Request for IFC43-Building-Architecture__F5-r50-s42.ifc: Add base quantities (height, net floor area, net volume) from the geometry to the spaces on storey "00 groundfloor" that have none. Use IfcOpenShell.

First a look at what the model holds.

```python
import ifcopenshell
import ifcopenshell.util.element
import ifcopenshell.util.unit

model = ifcopenshell.open("IFC43-Building-Architecture__F5-r50-s42.ifc")
print(model.schema)
for unit_type in ("LENGTHUNIT", "AREAUNIT", "VOLUMEUNIT"):
    print(unit_type, ifcopenshell.util.unit.calculate_unit_scale(model, unit_type))
storey = next(s for s in model.by_type("IfcBuildingStorey") if s.Name == "00 groundfloor")
spaces = [e for e in ifcopenshell.util.element.get_decomposition(storey) if e.is_a("IfcSpace")]
for e in sorted(spaces, key=lambda e: e.id()):
    print(e.id(), e.is_a(), e.Name, list(ifcopenshell.util.element.get_psets(e, qtos_only=True)), sep=" | ")
```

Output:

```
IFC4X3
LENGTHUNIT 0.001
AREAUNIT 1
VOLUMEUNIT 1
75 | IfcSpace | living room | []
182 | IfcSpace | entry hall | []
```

```python
import ifcopenshell
import ifcopenshell.api.pset
import ifcopenshell.geom
import ifcopenshell.util.element
import ifcopenshell.util.shape
import ifcopenshell.util.unit

model = ifcopenshell.open("IFC43-Building-Architecture__F5-r50-s42.ifc")
unit_scale = ifcopenshell.util.unit.calculate_unit_scale(model)
area_scale = ifcopenshell.util.unit.calculate_unit_scale(model, "AREAUNIT")
volume_scale = ifcopenshell.util.unit.calculate_unit_scale(model, "VOLUMEUNIT")
settings = ifcopenshell.geom.settings()

storey = next(s for s in model.by_type("IfcBuildingStorey") if s.Name == "00 groundfloor")
spaces = [e for e in ifcopenshell.util.element.get_decomposition(storey) if e.is_a("IfcSpace")]

for e in sorted(spaces, key=lambda e: e.id()):
    if ifcopenshell.util.element.get_psets(e, qtos_only=True, should_inherit=False):
        continue
    # Geometry comes back in metres, in the element's own axes.
    shape = ifcopenshell.geom.create_shape(settings, e)
    values = {
        "Height": ifcopenshell.util.shape.get_z(shape.geometry) / unit_scale,
        "NetFloorArea": ifcopenshell.util.shape.get_footprint_area(shape.geometry) / area_scale,
        "NetVolume": ifcopenshell.util.shape.get_volume(shape.geometry) / volume_scale,
    }
    qto = ifcopenshell.api.pset.add_qto(model, product=e, name="Qto_SpaceBaseQuantities")
    ifcopenshell.api.pset.edit_qto(model, qto=qto, properties=values)
    print(e.id(), {k: round(v, 3) for k, v in values.items()})

model.write("IFC43-Building-Architecture__F5-r50-s42-out.ifc")
```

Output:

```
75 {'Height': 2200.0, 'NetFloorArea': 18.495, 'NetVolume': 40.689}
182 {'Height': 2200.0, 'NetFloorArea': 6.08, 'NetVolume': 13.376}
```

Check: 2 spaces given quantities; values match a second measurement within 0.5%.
